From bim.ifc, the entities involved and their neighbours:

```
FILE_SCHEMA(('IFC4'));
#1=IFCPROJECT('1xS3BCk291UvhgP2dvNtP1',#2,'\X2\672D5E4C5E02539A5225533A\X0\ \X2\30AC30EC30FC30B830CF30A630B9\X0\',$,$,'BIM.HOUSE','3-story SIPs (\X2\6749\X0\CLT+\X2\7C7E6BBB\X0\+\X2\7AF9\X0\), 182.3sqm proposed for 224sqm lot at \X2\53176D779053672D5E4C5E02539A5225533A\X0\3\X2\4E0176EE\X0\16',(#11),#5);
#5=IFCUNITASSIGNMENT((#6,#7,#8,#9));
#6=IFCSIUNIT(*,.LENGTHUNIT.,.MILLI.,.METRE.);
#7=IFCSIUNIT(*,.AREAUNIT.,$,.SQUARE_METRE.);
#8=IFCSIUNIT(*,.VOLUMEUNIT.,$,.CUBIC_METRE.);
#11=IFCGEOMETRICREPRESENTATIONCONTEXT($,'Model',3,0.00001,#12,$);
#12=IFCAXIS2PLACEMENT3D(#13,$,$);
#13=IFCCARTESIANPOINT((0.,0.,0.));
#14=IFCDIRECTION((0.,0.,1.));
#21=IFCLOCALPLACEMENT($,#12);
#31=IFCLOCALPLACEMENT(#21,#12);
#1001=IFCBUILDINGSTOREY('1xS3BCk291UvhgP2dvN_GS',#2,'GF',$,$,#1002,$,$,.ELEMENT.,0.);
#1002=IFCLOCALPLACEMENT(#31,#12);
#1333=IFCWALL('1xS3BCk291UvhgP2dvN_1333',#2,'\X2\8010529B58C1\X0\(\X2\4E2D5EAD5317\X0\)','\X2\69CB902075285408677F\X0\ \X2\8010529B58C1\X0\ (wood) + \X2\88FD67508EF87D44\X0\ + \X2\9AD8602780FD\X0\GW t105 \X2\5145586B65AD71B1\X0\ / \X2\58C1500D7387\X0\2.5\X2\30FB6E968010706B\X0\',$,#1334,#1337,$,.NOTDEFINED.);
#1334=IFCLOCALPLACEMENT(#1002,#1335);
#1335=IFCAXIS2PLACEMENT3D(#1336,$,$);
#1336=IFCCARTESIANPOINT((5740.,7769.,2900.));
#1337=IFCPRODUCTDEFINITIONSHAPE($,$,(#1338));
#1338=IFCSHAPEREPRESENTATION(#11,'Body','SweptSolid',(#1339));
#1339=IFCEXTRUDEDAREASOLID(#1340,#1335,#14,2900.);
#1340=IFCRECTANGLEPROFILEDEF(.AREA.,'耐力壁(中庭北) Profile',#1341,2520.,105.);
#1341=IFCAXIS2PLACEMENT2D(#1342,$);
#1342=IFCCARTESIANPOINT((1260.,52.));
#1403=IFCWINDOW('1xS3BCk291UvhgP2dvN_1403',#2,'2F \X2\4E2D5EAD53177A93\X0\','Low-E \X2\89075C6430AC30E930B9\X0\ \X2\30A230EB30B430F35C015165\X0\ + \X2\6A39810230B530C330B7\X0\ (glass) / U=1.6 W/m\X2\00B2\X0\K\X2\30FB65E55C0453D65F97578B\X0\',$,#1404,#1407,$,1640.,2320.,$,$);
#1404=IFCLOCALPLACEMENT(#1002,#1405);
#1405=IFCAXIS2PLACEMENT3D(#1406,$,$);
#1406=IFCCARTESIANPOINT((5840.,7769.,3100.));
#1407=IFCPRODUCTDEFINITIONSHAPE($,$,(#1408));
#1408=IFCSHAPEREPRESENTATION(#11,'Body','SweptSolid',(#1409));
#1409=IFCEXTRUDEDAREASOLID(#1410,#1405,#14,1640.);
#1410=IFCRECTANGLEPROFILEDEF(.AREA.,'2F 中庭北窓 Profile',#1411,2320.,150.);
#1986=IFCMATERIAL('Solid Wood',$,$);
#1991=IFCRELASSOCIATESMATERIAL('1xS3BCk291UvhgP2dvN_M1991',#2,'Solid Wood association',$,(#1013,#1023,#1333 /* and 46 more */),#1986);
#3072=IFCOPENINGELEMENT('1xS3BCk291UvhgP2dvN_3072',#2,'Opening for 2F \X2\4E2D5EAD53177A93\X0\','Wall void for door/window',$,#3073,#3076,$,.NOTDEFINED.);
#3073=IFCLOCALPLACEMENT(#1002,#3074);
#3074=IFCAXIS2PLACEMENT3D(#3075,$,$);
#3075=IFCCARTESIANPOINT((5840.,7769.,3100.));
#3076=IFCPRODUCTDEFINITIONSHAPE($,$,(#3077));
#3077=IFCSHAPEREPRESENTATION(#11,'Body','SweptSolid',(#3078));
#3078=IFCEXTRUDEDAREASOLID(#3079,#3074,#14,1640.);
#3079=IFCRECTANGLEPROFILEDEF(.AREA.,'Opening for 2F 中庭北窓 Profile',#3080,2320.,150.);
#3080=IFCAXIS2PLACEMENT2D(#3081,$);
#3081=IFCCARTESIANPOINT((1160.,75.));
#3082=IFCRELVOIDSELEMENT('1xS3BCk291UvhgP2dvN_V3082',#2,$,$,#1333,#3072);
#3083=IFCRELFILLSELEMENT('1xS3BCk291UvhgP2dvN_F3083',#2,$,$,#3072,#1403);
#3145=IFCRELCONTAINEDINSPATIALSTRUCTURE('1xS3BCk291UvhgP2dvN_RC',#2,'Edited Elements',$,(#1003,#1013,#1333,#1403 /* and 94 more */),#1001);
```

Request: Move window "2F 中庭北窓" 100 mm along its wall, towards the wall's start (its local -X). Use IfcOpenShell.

```python
import ifcopenshell
import ifcopenshell.api.geometry
import ifcopenshell.util.placement
import ifcopenshell.util.unit

model = ifcopenshell.open("bim.ifc")
unit_scale = ifcopenshell.util.unit.calculate_unit_scale(model)

window = model.by_guid("1xS3BCk291UvhgP2dvN_1403")
opening = window.FillsVoids[0].RelatingOpeningElement
wall = opening.VoidsElements[0].RelatingBuildingElement

wall_matrix = ifcopenshell.util.placement.get_local_placement(wall.ObjectPlacement)
shift = wall_matrix[:3, 0] * -0.1 / unit_scale
before = ifcopenshell.util.placement.get_local_placement(window.ObjectPlacement)[:3, 3].copy()

# The window is not placed relative to its opening, so move both.
for product in (opening, window):
    matrix = ifcopenshell.util.placement.get_local_placement(product.ObjectPlacement)
    matrix[:3, 3] += shift
    ifcopenshell.api.geometry.edit_object_placement(model, product=product, matrix=matrix, is_si=False)

after = ifcopenshell.util.placement.get_local_placement(window.ObjectPlacement)[:3, 3]
print("window moved by", (after - before).round(3) + 0.0)

model.write("bim_v2.ifc")
```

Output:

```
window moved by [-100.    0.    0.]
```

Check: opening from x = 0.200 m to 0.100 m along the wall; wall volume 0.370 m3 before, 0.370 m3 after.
